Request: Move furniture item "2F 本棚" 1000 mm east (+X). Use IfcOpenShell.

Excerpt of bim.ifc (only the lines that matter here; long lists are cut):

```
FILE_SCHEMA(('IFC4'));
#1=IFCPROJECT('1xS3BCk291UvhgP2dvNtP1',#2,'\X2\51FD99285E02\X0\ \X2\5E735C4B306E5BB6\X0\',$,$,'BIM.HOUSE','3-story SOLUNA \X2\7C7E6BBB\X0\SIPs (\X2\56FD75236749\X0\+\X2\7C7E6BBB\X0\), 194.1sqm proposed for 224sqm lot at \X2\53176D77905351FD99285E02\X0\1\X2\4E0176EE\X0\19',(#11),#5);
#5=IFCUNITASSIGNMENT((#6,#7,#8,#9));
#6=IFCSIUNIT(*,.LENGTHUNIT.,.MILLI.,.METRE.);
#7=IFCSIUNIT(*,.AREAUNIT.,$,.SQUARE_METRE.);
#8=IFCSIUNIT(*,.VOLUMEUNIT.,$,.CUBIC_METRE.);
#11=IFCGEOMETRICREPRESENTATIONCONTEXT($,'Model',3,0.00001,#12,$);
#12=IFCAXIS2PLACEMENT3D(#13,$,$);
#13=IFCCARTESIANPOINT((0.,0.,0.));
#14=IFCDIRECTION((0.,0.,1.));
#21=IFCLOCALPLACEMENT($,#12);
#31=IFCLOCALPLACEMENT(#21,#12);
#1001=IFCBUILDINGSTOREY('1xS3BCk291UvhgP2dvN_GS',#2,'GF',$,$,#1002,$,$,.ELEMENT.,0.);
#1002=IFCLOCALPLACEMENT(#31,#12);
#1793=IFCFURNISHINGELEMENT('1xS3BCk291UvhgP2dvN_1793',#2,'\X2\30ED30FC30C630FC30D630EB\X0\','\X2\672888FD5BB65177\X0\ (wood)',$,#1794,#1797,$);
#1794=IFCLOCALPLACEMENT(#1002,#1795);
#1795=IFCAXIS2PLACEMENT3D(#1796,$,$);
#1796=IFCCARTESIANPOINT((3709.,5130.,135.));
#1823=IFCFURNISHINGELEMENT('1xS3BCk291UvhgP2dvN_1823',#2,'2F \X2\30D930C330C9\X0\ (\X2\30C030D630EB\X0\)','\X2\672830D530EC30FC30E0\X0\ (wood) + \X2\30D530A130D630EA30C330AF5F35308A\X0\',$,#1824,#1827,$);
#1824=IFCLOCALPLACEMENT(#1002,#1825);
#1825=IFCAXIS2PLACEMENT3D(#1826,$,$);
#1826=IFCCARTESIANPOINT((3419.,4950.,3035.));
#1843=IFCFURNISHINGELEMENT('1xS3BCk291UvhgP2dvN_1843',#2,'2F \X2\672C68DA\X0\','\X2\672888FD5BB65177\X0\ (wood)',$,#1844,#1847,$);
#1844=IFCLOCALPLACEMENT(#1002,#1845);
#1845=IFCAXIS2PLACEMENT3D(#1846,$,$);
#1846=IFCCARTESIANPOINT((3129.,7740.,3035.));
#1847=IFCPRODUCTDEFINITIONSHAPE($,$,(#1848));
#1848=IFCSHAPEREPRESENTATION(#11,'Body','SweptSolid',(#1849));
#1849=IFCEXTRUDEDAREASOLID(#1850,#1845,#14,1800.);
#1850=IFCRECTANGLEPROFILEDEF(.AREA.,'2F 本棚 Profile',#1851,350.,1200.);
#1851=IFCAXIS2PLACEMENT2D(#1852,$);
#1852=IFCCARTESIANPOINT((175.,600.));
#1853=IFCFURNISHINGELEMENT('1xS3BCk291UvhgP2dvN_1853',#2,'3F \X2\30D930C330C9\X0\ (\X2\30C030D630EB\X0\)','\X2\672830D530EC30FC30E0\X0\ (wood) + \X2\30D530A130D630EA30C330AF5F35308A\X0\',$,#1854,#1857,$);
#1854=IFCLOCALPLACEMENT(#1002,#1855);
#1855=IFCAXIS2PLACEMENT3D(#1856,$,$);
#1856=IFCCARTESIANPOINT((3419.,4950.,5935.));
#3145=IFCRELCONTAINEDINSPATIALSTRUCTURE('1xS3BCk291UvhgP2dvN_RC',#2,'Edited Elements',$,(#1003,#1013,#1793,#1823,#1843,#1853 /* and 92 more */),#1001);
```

```python
import ifcopenshell
import ifcopenshell.api.geometry
import ifcopenshell.util.placement
import ifcopenshell.util.unit

model = ifcopenshell.open("bim.ifc")
unit_scale = ifcopenshell.util.unit.calculate_unit_scale(model)

item = model.by_guid("1xS3BCk291UvhgP2dvN_1843")
matrix = ifcopenshell.util.placement.get_local_placement(item.ObjectPlacement)
matrix[0, 3] += 1 / unit_scale
ifcopenshell.api.geometry.edit_object_placement(model, product=item, matrix=matrix, is_si=False)

print(ifcopenshell.util.placement.get_local_placement(item.ObjectPlacement).round(3) + 0.0)

model.write("bim_edited.ifc")
```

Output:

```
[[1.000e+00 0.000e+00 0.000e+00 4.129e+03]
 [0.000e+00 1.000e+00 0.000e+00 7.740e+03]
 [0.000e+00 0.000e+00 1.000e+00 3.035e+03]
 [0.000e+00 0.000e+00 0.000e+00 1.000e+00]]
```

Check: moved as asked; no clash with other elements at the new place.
